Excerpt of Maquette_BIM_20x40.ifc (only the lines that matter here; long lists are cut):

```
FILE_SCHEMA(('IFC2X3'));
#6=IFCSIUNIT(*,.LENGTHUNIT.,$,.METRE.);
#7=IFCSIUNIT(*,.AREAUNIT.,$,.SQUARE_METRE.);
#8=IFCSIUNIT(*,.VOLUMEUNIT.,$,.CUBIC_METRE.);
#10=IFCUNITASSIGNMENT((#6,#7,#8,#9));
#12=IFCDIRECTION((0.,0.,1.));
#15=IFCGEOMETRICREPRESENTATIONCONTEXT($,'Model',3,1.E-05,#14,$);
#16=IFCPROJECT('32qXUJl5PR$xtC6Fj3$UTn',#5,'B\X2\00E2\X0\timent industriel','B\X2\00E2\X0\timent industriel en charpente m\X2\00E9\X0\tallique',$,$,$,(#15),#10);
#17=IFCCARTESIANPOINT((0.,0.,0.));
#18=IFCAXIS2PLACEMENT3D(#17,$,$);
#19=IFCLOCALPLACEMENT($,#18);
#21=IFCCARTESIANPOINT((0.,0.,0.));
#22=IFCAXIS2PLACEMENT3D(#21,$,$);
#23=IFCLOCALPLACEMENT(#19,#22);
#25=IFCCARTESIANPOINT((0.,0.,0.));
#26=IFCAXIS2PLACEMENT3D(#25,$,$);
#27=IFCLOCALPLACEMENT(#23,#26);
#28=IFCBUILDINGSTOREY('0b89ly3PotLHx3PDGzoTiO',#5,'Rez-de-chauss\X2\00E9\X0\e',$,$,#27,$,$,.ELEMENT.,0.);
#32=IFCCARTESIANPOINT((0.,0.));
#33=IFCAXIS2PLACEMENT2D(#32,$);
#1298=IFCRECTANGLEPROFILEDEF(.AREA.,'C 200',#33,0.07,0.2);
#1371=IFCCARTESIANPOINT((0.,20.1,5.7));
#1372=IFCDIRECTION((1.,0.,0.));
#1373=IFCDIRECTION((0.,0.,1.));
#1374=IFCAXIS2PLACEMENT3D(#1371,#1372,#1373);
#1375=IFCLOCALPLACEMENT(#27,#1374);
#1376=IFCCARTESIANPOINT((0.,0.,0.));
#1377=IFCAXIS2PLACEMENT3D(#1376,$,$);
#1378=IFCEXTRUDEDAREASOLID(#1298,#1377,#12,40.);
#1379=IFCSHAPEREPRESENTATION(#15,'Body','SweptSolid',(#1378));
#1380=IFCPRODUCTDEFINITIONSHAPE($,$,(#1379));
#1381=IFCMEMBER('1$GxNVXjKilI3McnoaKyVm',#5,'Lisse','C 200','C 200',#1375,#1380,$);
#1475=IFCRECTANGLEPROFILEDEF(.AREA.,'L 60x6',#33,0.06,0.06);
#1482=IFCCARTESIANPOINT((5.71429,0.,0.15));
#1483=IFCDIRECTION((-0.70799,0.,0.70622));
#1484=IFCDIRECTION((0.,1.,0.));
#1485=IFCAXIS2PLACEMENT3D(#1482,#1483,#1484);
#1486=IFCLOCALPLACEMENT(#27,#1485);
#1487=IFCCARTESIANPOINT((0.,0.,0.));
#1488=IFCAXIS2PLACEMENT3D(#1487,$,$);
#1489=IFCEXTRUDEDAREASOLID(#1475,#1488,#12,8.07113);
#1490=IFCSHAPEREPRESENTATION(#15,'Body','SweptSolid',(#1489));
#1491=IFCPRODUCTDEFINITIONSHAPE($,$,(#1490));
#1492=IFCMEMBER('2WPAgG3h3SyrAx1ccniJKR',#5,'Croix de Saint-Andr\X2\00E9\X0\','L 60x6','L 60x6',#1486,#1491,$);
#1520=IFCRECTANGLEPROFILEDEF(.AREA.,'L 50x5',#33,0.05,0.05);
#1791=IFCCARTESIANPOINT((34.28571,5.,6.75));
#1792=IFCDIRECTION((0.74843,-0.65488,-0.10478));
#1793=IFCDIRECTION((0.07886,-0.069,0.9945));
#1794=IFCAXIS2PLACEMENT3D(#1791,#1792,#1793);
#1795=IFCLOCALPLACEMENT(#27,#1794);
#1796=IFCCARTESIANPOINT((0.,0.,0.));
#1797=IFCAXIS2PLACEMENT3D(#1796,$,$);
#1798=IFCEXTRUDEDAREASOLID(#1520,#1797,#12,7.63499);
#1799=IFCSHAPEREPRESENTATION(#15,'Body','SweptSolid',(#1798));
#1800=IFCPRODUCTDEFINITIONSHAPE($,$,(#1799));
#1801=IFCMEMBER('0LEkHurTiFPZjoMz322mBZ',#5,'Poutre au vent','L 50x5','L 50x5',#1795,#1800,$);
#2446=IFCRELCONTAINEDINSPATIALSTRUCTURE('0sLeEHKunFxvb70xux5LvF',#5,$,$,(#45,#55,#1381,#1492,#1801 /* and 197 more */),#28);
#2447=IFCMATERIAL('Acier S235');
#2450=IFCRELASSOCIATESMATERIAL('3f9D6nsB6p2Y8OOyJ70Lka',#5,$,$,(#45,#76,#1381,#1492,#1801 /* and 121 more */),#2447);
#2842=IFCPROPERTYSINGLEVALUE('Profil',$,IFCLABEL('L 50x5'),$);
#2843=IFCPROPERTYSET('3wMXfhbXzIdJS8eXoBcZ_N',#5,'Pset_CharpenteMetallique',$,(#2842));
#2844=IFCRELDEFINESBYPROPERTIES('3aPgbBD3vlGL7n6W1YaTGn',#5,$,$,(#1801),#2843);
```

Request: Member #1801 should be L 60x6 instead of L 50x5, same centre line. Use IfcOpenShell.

```python
import ifcopenshell
import ifcopenshell.api.pset
import ifcopenshell.util.element

model = ifcopenshell.open("Maquette_BIM_20x40.ifc")

member = model.by_guid("0LEkHurTiFPZjoMz322mBZ")
source = next(p for p in model.by_type("IfcRectangleProfileDef") if p.ProfileName == "L 60x6")

body = next(r for r in member.Representation.Representations if r.RepresentationIdentifier == "Body")
solid = body.Items[0]
old_profile = solid.SweptArea

# Copy the section's sizes but keep this member's own profile position.
profile = ifcopenshell.util.element.copy(model, source)
profile.Position = old_profile.Position
solid.SweptArea = profile
if not model.get_total_inverses(old_profile):
    ifcopenshell.util.element.remove_deep2(model, old_profile)
member.Description = member.Description.replace("L 50x5", "L 60x6")
member.ObjectType = member.ObjectType.replace("L 50x5", "L 60x6")
pset = model.by_id(ifcopenshell.util.element.get_pset(member, "Pset_CharpenteMetallique", should_inherit=False)["id"])
ifcopenshell.api.pset.edit_pset(model, pset=pset, properties={"Profil": "L 60x6"})

print(solid.SweptArea)

model.write("Maquette_BIM_20x40_edited.ifc")
```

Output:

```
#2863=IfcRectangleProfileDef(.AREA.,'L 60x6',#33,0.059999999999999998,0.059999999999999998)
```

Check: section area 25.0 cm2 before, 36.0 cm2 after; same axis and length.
